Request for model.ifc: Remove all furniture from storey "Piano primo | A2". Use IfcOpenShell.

First a look at what the model holds.

```python
import ifcopenshell
import ifcopenshell.util.element

model = ifcopenshell.open("model.ifc")
print(model.schema)
storey = next(s for s in model.by_type("IfcBuildingStorey") if s.Name == "Piano primo | A2")
furniture = [e for e in ifcopenshell.util.element.get_decomposition(storey) if e.is_a("IfcFurnishingElement")]
seen = {}
for e in furniture:
    element_type = ifcopenshell.util.element.get_type(e)
    name = element_type.Name if element_type not in (None, e) else None
    seen[name] = seen.get(name, 0) + 1
for name, count in sorted(seen.items(), key=str):
    print(count, "x", name)
```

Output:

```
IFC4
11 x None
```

```python
import ifcopenshell
import ifcopenshell.api.root
import ifcopenshell.util.element

model = ifcopenshell.open("model.ifc")

storey = next(s for s in model.by_type("IfcBuildingStorey") if s.Name == "Piano primo | A2")
furniture = [e for e in ifcopenshell.util.element.get_decomposition(storey) if e.is_a("IfcFurnishingElement")]

for e in furniture:
    ifcopenshell.api.root.remove_product(model, product=e)
print(len(furniture), "removed")

model.write("model_updated.ifc")
```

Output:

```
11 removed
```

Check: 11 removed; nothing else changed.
